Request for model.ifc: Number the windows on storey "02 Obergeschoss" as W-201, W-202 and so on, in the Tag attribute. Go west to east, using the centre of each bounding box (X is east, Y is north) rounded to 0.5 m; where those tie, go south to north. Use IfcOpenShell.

First a look at what the model holds.

```python
import ifcopenshell
import ifcopenshell.util.element
import ifcopenshell.util.placement

model = ifcopenshell.open("model.ifc")
print(model.schema)
storey = next(s for s in model.by_type("IfcBuildingStorey") if s.Name == "02 Obergeschoss")
windows = [e for e in ifcopenshell.util.element.get_decomposition(storey) if e.is_a("IfcWindow")]
for e in sorted(windows, key=lambda e: e.id()):
    origin = ifcopenshell.util.placement.get_local_placement(e.ObjectPlacement)[:3, 3]
    print(e.id(), e.Tag, e.Name, origin.round(2) + 0.0, sep=" | ")
```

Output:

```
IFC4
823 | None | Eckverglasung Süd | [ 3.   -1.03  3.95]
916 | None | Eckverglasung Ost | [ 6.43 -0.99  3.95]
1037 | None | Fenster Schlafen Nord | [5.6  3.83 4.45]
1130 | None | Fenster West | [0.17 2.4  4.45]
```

```python
import ifcopenshell
import ifcopenshell.geom
import ifcopenshell.util.element
import ifcopenshell.util.shape

model = ifcopenshell.open("model.ifc")
settings = ifcopenshell.geom.settings()
settings.set("use-world-coords", True)


def centre(element):
    shape = ifcopenshell.geom.create_shape(settings, element)
    return ifcopenshell.util.shape.get_bbox_centroid(shape.geometry)


storey = next(s for s in model.by_type("IfcBuildingStorey") if s.Name == "02 Obergeschoss")
windows = [e for e in ifcopenshell.util.element.get_decomposition(storey) if e.is_a("IfcWindow")]

# Insertion points can sit at a corner or the storey origin, so sort by the geometry (in metres).
centres = {e: centre(e) for e in windows}
windows.sort(key=lambda e: (round(centres[e][0] / 0.5), centres[e][1]))

for i, e in enumerate(windows, start=1):
    number = f"W-2{i:02d}"
    e.Tag = number
    print(e.id(), number)

model.write("model-out.ifc")
```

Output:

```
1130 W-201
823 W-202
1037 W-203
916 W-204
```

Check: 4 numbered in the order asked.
